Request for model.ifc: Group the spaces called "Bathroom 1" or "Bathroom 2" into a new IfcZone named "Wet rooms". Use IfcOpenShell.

First a look at what the model holds.

```python
import ifcopenshell

model = ifcopenshell.open("model.ifc")
print(model.schema)
seen = {}
for space in model.by_type("IfcSpace"):
    seen[space.LongName] = seen.get(space.LongName, 0) + 1
for name, count in sorted(seen.items(), key=str):
    print(count, "x", name)
print("zones:", [z.Name for z in model.by_type("IfcZone")][:20])
```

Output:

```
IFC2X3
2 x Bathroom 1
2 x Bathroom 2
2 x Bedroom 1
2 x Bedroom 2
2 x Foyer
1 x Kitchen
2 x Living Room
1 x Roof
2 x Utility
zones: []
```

```python
import ifcopenshell
import ifcopenshell.api.group
import ifcopenshell.api.root

model = ifcopenshell.open("model.ifc")

names = {"Bathroom 1", "Bathroom 2"}
spaces = [s for s in model.by_type("IfcSpace") if s.LongName in names]

zone = ifcopenshell.api.root.create_entity(model, ifc_class="IfcZone", name="Wet rooms")
ifcopenshell.api.group.assign_group(model, products=spaces, group=zone)
print(len(spaces), "spaces in", zone.Name)

model.write("model_v2.ifc")
```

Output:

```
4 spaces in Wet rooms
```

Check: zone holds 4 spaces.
